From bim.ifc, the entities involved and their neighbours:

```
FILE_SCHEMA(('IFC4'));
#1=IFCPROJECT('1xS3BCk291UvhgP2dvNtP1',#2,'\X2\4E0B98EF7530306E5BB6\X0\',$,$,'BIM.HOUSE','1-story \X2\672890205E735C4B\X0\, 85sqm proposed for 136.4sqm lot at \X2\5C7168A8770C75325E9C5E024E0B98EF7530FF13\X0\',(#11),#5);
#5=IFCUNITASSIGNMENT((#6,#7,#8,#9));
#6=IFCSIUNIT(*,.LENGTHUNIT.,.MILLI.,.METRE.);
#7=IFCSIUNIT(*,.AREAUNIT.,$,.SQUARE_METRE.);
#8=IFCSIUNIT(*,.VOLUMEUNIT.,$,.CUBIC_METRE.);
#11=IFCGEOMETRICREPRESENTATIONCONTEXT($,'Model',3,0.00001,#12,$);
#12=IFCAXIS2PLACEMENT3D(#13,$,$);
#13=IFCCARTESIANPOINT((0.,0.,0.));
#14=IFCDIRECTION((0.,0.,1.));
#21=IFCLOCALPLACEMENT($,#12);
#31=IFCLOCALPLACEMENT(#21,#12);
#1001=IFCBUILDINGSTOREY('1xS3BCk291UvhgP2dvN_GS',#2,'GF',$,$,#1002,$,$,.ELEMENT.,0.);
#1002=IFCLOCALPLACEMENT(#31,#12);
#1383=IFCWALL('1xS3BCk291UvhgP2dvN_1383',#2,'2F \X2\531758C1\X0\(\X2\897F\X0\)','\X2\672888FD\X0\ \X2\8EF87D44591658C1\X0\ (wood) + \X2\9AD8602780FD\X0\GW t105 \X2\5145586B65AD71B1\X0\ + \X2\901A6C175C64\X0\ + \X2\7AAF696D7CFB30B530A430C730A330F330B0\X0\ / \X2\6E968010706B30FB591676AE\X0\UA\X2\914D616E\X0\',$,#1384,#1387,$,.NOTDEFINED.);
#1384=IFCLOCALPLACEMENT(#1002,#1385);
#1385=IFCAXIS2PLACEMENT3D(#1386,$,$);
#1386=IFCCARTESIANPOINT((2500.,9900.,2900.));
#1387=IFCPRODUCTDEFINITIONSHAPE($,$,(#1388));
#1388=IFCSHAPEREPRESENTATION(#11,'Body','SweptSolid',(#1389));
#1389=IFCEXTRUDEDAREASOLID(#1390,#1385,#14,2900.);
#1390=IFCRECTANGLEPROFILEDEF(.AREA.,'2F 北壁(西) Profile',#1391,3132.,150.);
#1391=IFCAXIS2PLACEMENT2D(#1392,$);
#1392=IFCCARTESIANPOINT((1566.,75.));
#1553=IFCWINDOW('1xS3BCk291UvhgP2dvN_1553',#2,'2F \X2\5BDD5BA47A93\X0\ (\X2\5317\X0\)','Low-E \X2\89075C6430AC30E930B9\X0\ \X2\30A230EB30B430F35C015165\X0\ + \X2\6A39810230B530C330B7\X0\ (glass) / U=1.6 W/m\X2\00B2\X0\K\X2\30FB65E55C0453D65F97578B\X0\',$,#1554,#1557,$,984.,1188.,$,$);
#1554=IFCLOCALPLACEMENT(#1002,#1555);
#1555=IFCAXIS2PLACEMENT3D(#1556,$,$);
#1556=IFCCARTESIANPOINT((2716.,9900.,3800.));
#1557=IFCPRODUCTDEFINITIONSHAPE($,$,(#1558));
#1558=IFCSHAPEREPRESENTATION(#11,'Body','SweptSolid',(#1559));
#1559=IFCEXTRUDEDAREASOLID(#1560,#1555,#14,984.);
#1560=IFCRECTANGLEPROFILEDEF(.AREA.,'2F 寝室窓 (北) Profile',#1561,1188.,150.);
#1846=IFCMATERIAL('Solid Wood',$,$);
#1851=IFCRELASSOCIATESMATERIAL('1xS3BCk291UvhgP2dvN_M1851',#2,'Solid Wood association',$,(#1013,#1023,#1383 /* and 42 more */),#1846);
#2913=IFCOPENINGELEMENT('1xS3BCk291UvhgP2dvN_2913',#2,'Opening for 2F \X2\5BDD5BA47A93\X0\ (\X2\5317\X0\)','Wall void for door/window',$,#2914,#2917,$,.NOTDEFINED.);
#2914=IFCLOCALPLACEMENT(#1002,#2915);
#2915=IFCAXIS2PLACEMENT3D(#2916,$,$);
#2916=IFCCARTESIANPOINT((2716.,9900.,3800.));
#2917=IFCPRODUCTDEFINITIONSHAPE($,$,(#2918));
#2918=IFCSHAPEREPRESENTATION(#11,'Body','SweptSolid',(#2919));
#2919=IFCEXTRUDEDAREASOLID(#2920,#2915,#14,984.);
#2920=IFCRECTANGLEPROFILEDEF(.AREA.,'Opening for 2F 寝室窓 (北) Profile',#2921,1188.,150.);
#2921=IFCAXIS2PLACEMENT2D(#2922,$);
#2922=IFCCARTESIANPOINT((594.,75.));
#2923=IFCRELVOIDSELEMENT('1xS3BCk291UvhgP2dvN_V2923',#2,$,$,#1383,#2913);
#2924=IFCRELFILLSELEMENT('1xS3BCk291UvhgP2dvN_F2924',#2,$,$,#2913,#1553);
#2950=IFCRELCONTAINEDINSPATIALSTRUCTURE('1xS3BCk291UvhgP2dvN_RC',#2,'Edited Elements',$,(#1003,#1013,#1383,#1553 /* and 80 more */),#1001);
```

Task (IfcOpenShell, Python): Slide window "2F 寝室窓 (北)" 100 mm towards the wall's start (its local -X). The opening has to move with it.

```python
import ifcopenshell
import ifcopenshell.api.geometry
import ifcopenshell.util.placement
import ifcopenshell.util.unit

model = ifcopenshell.open("bim.ifc")
unit_scale = ifcopenshell.util.unit.calculate_unit_scale(model)

window = model.by_guid("1xS3BCk291UvhgP2dvN_1553")
opening = window.FillsVoids[0].RelatingOpeningElement
wall = opening.VoidsElements[0].RelatingBuildingElement

wall_matrix = ifcopenshell.util.placement.get_local_placement(wall.ObjectPlacement)
shift = wall_matrix[:3, 0] * -0.1 / unit_scale
before = ifcopenshell.util.placement.get_local_placement(window.ObjectPlacement)[:3, 3].copy()

# The window is not placed relative to its opening, so move both.
for product in (opening, window):
    matrix = ifcopenshell.util.placement.get_local_placement(product.ObjectPlacement)
    matrix[:3, 3] += shift
    ifcopenshell.api.geometry.edit_object_placement(model, product=product, matrix=matrix, is_si=False)

after = ifcopenshell.util.placement.get_local_placement(window.ObjectPlacement)[:3, 3]
print("window moved by", (after - before).round(3) + 0.0)

model.write("bim_v2.ifc")
```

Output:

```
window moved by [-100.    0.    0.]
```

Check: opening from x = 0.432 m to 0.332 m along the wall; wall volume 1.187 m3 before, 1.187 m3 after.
